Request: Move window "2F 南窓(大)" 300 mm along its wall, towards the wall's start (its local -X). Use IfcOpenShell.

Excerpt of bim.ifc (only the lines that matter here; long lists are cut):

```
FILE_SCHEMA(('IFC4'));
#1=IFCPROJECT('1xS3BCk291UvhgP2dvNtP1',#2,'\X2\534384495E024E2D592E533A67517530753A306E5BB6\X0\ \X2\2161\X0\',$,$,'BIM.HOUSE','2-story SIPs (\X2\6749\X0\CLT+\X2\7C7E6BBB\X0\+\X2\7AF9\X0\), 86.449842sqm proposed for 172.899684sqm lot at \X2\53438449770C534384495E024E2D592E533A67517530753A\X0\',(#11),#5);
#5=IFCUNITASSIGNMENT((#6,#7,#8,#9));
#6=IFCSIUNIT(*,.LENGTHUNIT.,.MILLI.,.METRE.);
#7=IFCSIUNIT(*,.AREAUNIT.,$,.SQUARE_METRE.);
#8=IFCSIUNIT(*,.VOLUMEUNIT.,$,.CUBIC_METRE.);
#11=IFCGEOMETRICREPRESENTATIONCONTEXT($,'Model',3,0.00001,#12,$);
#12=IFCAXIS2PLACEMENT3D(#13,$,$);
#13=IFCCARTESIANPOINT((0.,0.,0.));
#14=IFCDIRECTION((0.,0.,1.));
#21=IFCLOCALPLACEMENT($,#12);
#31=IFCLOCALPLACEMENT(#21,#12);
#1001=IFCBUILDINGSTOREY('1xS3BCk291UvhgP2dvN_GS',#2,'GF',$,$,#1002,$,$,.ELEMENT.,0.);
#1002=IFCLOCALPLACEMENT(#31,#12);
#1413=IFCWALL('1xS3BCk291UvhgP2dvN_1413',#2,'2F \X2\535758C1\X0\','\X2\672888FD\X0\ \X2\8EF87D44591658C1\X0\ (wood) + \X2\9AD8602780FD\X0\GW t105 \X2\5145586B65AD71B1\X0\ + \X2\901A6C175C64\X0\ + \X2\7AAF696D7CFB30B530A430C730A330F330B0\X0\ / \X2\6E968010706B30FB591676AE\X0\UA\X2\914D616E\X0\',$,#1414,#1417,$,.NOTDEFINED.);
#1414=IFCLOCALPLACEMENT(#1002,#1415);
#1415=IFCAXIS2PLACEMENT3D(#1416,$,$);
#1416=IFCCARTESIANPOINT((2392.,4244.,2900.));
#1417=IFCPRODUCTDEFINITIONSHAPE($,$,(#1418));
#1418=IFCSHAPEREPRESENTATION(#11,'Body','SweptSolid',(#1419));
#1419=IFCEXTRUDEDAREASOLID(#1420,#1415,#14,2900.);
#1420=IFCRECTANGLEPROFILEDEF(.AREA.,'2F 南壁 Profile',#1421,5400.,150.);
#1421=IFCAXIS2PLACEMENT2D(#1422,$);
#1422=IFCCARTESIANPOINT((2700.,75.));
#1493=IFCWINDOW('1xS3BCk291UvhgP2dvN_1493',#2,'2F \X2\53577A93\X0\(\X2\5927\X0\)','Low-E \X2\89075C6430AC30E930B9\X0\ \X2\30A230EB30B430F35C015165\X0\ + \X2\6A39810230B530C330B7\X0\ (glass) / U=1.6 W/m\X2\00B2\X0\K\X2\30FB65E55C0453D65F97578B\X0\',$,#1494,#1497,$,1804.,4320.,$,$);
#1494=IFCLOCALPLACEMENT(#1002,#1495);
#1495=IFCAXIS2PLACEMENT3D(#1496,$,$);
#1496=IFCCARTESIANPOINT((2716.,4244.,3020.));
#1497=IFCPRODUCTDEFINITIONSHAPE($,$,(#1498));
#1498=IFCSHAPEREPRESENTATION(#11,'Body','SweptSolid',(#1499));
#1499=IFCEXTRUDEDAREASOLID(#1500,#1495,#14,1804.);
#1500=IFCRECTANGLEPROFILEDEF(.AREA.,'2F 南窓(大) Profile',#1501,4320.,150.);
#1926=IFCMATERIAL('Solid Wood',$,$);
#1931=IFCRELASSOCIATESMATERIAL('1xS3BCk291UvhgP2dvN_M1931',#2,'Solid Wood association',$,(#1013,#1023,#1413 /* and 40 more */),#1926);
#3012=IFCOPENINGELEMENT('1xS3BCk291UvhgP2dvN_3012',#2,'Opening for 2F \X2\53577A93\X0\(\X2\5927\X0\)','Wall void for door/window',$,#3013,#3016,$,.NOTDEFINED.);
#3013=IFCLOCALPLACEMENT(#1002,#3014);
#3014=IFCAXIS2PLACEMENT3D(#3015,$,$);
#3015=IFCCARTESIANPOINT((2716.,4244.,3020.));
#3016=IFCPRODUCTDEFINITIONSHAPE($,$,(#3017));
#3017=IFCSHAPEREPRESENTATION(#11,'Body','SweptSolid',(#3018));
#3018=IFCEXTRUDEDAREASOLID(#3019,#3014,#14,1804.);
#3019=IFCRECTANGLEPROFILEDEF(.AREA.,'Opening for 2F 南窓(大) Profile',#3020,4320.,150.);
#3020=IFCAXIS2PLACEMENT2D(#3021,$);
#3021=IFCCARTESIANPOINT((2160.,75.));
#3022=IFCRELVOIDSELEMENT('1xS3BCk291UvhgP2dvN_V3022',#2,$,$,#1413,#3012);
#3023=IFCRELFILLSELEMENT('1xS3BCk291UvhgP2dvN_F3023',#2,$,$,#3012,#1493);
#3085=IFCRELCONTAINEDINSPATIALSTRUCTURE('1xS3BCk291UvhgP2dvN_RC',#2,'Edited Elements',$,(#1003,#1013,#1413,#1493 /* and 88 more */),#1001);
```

```python
import ifcopenshell
import ifcopenshell.api.geometry
import ifcopenshell.util.placement
import ifcopenshell.util.unit

model = ifcopenshell.open("bim.ifc")
unit_scale = ifcopenshell.util.unit.calculate_unit_scale(model)

window = model.by_id(1493)
opening = window.FillsVoids[0].RelatingOpeningElement
wall = opening.VoidsElements[0].RelatingBuildingElement

wall_matrix = ifcopenshell.util.placement.get_local_placement(wall.ObjectPlacement)
shift = wall_matrix[:3, 0] * -0.3 / unit_scale
before = ifcopenshell.util.placement.get_local_placement(window.ObjectPlacement)[:3, 3].copy()

# The window is not placed relative to its opening, so move both.
for product in (opening, window):
    matrix = ifcopenshell.util.placement.get_local_placement(product.ObjectPlacement)
    matrix[:3, 3] += shift
    ifcopenshell.api.geometry.edit_object_placement(model, product=product, matrix=matrix, is_si=False)

after = ifcopenshell.util.placement.get_local_placement(window.ObjectPlacement)[:3, 3]
print("window moved by", (after - before).round(3) + 0.0)

model.write("bim_updated.ifc")
```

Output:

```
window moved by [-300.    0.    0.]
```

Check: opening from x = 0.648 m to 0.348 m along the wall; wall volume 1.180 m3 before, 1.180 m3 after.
